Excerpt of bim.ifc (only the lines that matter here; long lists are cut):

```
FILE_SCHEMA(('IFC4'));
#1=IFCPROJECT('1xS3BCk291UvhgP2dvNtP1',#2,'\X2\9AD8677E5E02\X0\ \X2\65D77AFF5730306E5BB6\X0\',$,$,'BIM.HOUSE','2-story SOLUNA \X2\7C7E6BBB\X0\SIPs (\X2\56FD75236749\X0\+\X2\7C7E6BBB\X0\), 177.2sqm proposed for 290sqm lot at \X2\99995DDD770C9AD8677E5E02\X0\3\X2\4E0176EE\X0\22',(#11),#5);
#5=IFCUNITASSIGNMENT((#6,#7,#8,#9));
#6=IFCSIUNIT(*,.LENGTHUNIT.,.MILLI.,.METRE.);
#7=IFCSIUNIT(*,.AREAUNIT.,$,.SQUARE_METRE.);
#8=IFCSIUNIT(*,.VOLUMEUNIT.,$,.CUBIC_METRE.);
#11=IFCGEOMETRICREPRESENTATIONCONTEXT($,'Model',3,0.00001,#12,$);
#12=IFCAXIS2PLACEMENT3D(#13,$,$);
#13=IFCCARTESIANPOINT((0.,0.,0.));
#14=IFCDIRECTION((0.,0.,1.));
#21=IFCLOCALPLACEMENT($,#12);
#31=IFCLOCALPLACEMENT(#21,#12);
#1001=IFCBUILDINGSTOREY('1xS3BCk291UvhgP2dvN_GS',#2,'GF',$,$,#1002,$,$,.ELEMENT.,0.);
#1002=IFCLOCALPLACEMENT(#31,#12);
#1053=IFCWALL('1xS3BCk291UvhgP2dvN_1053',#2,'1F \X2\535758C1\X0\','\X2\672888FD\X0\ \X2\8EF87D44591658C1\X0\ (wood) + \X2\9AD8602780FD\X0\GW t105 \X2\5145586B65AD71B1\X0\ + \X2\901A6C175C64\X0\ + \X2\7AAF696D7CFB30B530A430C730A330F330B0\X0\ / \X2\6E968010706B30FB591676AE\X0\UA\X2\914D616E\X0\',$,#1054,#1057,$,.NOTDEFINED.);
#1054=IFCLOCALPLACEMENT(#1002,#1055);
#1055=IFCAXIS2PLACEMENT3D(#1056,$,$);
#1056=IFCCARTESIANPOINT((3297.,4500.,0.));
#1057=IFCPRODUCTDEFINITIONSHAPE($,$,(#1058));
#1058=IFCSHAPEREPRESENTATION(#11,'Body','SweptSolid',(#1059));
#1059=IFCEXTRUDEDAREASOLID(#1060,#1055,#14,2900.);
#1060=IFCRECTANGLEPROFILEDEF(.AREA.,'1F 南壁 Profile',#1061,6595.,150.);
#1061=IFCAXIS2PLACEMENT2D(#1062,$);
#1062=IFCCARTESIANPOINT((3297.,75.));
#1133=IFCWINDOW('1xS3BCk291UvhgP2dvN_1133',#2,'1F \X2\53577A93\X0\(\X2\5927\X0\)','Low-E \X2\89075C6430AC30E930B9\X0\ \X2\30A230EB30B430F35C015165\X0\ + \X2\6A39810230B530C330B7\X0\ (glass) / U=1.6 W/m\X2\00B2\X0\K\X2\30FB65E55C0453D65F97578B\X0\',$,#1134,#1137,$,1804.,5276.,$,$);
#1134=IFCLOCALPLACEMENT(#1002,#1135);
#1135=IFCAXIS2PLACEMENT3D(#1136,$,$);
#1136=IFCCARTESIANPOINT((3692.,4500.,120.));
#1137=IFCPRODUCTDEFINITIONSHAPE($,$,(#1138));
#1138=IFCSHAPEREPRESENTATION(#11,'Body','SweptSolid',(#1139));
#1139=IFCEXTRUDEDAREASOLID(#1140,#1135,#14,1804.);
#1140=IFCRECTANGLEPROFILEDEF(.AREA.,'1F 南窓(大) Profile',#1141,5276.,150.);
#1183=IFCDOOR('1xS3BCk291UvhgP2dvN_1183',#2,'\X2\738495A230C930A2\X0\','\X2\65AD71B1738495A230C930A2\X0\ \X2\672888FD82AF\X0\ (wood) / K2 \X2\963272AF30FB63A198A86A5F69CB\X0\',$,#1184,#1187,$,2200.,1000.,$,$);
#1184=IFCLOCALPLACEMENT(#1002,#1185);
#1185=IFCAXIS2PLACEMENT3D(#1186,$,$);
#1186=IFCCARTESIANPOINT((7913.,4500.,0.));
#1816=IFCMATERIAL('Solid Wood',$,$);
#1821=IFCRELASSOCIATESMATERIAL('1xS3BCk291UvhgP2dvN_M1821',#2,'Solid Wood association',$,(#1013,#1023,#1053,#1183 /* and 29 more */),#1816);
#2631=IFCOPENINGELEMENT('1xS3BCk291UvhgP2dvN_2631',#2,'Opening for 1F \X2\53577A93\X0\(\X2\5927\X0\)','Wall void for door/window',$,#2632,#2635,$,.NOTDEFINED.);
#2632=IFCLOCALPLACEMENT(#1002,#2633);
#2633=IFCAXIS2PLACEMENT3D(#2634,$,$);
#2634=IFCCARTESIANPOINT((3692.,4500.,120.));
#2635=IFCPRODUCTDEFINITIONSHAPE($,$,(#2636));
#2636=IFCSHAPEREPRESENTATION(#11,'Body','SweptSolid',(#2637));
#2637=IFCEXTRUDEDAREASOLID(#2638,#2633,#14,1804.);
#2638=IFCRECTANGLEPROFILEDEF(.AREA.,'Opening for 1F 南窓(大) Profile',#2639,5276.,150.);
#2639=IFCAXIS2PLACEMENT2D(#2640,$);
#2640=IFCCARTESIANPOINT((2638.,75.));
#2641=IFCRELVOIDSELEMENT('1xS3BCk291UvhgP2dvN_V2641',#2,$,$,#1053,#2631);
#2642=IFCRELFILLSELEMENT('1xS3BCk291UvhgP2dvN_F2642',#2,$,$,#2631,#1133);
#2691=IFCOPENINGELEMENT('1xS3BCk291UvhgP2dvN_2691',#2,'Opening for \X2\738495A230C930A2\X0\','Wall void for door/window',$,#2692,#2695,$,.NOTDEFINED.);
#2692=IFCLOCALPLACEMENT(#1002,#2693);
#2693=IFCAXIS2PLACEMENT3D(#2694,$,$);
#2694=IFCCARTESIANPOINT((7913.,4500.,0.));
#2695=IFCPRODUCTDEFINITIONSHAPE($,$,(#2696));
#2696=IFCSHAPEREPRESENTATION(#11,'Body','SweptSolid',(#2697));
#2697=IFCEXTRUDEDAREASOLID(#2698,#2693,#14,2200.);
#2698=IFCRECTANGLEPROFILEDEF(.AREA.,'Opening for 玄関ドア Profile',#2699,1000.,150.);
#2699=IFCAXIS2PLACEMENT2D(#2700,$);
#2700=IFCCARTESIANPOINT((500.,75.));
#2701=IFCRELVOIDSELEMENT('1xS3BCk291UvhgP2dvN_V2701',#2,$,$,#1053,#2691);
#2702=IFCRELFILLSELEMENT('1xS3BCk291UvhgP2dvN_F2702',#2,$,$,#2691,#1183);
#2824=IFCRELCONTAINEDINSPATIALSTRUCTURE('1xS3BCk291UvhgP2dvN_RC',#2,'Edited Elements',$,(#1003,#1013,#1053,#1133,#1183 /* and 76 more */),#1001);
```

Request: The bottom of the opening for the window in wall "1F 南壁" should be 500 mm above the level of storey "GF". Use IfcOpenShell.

```python
import numpy as np
import ifcopenshell
import ifcopenshell.api.geometry
import ifcopenshell.geom
import ifcopenshell.util.element
import ifcopenshell.util.placement
import ifcopenshell.util.shape
import ifcopenshell.util.unit

model = ifcopenshell.open("bim.ifc")
unit_scale = ifcopenshell.util.unit.calculate_unit_scale(model)

window = model.by_guid("1xS3BCk291UvhgP2dvN_1133")
opening = window.FillsVoids[0].RelatingOpeningElement
storey = ifcopenshell.util.element.get_container(window, ifc_class="IfcBuildingStorey")
level = ifcopenshell.util.placement.get_local_placement(storey.ObjectPlacement)[2, 3]

# The opening's origin need not be at the sill, so measure its lowest point.
shape = ifcopenshell.geom.create_shape(ifcopenshell.geom.settings(), opening)
bottom = ifcopenshell.util.shape.get_shape_bottom_elevation(shape, shape.geometry) / unit_scale
dz = level + 0.5 / unit_scale - bottom

shift = np.array([0.0, 0.0, dz])
# The window is not placed relative to its opening, so move both.
for product in (opening, window):
    matrix = ifcopenshell.util.placement.get_local_placement(product.ObjectPlacement)
    matrix[:3, 3] += shift
    ifcopenshell.api.geometry.edit_object_placement(model, product=product, matrix=matrix, is_si=False)

print(f"moved by {dz * unit_scale:+.3f} m")

model.write("bim_edited.ifc")
```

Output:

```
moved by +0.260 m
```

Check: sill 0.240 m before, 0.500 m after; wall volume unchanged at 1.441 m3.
